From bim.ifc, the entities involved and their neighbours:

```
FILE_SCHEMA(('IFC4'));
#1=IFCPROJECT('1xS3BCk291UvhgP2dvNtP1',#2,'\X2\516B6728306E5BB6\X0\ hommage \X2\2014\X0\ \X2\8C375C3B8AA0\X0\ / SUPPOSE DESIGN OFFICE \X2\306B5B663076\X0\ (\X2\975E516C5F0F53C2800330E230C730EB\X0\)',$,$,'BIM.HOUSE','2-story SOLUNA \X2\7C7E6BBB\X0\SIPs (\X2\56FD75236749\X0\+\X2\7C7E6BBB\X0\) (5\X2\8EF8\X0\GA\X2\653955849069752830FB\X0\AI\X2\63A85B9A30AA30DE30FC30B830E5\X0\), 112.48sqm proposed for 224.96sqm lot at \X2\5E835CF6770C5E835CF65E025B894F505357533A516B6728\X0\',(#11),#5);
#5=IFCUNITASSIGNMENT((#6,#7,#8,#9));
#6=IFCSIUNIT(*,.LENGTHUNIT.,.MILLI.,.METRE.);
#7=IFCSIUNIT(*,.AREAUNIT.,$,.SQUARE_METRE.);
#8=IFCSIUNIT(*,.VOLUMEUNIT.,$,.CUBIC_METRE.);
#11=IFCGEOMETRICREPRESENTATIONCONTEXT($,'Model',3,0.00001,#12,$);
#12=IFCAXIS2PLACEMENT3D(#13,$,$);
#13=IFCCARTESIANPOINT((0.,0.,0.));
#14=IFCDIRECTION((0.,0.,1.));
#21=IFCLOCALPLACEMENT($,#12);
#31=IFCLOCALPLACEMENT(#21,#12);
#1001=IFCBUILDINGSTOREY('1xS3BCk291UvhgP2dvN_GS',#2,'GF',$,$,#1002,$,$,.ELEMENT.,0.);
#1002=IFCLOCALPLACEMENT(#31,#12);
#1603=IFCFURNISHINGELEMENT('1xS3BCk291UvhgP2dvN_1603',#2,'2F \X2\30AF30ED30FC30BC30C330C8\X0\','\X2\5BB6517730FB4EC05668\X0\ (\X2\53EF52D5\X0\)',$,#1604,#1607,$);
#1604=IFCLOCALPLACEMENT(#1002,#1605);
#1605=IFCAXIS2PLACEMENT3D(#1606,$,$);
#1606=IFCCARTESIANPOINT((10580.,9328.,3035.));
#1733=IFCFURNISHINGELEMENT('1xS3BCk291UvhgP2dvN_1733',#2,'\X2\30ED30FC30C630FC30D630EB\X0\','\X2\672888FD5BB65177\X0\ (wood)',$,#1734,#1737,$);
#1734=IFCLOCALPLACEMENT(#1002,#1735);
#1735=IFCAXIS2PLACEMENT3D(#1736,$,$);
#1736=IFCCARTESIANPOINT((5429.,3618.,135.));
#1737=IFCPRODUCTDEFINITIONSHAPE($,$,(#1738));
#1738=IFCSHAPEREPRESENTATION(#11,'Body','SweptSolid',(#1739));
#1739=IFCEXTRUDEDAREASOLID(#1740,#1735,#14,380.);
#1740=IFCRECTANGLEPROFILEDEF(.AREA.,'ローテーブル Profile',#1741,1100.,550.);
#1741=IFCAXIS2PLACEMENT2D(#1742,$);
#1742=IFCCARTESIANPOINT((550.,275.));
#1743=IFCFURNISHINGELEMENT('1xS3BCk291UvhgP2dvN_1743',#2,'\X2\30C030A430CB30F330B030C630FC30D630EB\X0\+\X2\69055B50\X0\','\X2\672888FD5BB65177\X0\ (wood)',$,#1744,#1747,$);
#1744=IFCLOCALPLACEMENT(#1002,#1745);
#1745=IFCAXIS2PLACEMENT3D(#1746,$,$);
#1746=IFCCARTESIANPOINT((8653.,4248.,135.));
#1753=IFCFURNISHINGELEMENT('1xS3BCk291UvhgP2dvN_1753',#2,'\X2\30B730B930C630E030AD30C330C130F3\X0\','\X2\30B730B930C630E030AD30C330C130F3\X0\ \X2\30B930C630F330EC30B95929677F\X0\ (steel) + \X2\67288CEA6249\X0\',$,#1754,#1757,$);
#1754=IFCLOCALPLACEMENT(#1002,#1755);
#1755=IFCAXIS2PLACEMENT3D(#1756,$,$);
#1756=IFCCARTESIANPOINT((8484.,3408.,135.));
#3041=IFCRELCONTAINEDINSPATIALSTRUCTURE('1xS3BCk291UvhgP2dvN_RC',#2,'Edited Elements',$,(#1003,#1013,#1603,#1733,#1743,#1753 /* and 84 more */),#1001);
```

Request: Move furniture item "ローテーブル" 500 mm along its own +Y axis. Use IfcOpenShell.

```python
import ifcopenshell
import ifcopenshell.api.geometry
import ifcopenshell.util.placement

model = ifcopenshell.open("bim.ifc")

item = model.by_guid("1xS3BCk291UvhgP2dvN_1733")
matrix = ifcopenshell.util.placement.get_local_placement(item.ObjectPlacement)
matrix[:3, 3] += matrix[:3, 1] * 500.0
ifcopenshell.api.geometry.edit_object_placement(model, product=item, matrix=matrix, is_si=False)

print(ifcopenshell.util.placement.get_local_placement(item.ObjectPlacement).round(3) + 0.0)

model.write("bim_v2.ifc")
```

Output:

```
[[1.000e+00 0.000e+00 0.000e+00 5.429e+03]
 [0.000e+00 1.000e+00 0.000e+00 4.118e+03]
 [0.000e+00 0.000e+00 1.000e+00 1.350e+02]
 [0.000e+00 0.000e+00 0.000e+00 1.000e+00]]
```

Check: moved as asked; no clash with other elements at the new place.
